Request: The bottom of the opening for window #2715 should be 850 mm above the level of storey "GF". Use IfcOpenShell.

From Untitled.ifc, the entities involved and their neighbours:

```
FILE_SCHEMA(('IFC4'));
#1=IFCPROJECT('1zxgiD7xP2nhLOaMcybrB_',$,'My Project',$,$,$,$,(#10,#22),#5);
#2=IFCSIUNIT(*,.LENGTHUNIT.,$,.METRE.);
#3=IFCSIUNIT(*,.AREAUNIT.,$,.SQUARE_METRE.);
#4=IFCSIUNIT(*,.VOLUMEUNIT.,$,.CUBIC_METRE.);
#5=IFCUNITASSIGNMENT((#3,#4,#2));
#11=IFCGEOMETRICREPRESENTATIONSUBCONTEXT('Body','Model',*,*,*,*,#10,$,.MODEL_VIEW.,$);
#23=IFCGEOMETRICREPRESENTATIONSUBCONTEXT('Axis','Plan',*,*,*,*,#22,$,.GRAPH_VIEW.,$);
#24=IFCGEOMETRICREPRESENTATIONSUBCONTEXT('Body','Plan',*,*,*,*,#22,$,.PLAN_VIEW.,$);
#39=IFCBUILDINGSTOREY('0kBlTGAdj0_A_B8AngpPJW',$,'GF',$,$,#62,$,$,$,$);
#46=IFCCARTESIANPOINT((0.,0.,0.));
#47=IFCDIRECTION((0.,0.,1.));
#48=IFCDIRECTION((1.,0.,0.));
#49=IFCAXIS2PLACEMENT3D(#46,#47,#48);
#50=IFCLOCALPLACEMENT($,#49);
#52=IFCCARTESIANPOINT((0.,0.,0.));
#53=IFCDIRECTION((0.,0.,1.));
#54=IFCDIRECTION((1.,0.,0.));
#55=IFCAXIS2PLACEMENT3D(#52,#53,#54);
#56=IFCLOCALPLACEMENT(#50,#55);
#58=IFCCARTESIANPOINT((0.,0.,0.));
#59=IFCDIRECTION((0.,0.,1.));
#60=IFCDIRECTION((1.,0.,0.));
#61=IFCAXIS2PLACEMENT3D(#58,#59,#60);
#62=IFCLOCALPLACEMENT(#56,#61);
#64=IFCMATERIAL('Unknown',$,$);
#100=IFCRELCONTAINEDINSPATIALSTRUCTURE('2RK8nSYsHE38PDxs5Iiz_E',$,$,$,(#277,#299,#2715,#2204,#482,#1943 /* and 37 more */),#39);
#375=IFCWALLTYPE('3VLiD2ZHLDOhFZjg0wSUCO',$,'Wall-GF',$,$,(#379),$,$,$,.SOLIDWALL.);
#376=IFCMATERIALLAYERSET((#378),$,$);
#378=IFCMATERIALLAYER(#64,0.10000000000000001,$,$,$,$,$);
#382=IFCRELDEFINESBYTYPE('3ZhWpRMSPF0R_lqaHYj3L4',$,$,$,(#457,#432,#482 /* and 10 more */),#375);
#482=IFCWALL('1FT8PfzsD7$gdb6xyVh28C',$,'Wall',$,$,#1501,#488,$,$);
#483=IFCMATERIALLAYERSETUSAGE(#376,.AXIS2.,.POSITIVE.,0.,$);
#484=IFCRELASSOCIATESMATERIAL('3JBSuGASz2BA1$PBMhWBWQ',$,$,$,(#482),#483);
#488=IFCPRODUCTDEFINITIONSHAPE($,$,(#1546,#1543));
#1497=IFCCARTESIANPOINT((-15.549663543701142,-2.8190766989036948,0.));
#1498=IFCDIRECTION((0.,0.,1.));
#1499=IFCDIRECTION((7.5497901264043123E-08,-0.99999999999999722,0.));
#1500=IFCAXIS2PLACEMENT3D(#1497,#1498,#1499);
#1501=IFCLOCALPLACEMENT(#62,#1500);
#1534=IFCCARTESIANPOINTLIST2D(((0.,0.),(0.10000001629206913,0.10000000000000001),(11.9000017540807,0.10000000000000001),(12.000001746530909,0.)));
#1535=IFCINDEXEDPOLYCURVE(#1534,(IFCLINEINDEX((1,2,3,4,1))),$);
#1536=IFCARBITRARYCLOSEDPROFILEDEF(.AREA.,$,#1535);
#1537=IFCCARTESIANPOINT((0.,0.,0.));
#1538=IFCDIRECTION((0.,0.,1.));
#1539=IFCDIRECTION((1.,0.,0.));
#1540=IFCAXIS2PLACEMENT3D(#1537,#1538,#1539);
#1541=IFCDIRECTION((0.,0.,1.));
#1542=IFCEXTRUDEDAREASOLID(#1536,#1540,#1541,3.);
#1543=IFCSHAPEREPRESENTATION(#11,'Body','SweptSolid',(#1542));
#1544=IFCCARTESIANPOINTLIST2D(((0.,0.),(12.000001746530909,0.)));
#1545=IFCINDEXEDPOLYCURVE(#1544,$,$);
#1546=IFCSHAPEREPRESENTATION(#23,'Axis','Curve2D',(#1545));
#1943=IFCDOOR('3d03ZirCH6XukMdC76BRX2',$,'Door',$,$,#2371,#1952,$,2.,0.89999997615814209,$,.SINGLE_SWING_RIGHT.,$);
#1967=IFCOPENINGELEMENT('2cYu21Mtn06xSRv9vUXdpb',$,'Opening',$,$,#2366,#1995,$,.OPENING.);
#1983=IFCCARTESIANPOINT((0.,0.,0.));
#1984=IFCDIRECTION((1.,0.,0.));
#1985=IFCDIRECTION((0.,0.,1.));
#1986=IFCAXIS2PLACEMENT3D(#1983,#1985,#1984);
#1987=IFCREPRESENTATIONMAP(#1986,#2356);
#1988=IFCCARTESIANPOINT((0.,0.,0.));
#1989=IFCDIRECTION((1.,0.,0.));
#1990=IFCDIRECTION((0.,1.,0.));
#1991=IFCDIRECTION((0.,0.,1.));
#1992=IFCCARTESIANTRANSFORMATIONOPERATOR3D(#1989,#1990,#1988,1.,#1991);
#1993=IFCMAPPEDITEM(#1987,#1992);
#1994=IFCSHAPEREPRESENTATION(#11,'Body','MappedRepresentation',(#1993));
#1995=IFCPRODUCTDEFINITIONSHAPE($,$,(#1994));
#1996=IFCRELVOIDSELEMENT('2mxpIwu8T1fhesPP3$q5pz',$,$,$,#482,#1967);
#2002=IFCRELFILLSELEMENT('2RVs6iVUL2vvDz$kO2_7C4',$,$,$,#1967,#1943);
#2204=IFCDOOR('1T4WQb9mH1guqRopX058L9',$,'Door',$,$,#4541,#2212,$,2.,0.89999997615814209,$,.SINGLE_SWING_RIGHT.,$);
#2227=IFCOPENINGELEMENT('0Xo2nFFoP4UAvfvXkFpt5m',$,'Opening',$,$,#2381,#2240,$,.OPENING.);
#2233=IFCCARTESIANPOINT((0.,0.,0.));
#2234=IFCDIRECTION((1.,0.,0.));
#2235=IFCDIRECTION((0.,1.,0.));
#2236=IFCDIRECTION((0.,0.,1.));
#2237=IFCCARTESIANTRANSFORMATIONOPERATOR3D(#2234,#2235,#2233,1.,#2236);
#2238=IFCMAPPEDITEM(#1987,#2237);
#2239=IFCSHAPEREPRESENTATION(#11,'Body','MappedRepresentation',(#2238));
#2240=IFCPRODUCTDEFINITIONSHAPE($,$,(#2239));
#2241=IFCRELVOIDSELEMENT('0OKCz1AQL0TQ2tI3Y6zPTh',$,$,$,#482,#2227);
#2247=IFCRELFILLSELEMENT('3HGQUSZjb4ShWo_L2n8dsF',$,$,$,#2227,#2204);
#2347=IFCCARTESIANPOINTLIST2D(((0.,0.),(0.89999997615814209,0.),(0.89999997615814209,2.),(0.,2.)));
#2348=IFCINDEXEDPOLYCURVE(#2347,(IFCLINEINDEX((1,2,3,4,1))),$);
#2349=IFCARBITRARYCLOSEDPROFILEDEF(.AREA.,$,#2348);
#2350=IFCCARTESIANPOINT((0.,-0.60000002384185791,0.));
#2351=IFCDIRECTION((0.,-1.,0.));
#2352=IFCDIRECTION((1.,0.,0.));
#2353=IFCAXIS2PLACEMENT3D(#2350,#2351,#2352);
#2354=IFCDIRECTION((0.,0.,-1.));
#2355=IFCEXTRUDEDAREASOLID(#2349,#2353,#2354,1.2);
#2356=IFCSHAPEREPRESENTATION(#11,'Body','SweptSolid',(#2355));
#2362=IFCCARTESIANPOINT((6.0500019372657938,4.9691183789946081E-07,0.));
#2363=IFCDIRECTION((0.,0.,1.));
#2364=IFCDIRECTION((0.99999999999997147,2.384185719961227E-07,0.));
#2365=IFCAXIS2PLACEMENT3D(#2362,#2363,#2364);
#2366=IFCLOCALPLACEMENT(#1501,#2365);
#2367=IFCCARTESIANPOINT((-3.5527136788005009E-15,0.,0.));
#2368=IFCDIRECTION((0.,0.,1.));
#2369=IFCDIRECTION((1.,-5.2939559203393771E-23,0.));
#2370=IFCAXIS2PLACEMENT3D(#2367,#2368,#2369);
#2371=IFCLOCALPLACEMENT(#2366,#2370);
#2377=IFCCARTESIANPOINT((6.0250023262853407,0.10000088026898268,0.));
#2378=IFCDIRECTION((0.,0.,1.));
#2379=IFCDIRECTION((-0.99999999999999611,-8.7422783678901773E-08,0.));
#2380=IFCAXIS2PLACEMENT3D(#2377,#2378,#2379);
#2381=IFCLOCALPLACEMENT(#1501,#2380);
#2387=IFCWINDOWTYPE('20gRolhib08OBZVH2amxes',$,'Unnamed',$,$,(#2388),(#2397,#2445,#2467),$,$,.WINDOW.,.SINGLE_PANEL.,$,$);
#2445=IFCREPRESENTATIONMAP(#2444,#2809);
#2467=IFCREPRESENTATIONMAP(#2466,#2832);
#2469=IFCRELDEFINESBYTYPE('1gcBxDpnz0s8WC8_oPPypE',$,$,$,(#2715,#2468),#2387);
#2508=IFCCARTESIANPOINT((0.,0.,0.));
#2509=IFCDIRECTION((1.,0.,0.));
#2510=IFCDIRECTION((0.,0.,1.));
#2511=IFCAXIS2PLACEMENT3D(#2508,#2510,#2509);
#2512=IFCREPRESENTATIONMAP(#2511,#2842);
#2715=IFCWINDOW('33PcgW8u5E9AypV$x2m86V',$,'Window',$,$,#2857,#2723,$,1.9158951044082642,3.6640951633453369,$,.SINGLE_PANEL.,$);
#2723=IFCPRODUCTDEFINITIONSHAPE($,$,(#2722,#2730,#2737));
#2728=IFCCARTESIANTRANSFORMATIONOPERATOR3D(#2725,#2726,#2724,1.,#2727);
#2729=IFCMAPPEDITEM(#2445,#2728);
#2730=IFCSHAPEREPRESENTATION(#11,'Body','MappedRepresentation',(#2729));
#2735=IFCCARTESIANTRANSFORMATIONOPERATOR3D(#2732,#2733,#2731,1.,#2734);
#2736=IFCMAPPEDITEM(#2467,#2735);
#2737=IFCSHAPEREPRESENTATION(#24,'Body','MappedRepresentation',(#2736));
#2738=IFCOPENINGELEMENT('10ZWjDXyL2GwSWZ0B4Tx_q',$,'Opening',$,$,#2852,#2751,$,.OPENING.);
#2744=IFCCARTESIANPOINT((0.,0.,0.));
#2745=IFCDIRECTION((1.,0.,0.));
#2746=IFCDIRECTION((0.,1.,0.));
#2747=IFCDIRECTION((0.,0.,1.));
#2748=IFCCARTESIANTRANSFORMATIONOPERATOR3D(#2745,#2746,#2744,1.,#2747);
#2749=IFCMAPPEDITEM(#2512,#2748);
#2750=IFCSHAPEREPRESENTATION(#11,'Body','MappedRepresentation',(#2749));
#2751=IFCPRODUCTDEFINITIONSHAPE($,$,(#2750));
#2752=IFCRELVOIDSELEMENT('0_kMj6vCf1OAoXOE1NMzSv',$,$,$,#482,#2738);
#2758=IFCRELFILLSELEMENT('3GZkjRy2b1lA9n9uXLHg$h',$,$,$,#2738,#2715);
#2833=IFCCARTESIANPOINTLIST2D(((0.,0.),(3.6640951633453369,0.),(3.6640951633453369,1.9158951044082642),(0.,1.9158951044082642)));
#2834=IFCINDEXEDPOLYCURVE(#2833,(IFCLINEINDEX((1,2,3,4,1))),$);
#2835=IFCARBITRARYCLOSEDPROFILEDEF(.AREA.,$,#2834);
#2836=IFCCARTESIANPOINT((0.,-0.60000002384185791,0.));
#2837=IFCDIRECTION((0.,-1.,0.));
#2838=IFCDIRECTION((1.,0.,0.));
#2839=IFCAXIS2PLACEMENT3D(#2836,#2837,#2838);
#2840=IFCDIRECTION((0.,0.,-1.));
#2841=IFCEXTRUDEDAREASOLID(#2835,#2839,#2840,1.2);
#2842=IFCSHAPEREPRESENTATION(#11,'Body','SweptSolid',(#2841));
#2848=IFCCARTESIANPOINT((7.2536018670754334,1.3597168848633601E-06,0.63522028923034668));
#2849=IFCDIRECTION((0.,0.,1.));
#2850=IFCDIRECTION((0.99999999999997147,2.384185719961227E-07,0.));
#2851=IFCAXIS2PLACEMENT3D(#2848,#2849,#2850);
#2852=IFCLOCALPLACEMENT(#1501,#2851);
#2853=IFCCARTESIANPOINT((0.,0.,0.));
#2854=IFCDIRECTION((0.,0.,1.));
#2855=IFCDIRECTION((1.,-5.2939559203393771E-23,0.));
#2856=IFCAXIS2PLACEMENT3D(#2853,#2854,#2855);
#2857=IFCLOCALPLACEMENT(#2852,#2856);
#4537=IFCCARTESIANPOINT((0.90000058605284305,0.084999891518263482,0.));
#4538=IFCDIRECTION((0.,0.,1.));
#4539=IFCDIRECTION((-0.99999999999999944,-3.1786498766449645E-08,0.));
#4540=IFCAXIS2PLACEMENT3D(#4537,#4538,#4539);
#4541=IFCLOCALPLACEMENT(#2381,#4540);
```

```python
import numpy as np
import ifcopenshell
import ifcopenshell.api.geometry
import ifcopenshell.geom
import ifcopenshell.util.element
import ifcopenshell.util.placement
import ifcopenshell.util.shape
import ifcopenshell.util.unit

model = ifcopenshell.open("Untitled.ifc")
unit_scale = ifcopenshell.util.unit.calculate_unit_scale(model)

window = model.by_guid("33PcgW8u5E9AypV$x2m86V")
opening = window.FillsVoids[0].RelatingOpeningElement
storey = ifcopenshell.util.element.get_container(window, ifc_class="IfcBuildingStorey")
level = ifcopenshell.util.placement.get_local_placement(storey.ObjectPlacement)[2, 3]

# The opening's origin need not be at the sill, so measure its lowest point.
shape = ifcopenshell.geom.create_shape(ifcopenshell.geom.settings(), opening)
bottom = ifcopenshell.util.shape.get_shape_bottom_elevation(shape, shape.geometry) / unit_scale
dz = level + 0.85 / unit_scale - bottom

shift = np.array([0.0, 0.0, dz])
# The window is placed relative to its opening, so it follows when the opening moves.
matrix = ifcopenshell.util.placement.get_local_placement(opening.ObjectPlacement)
matrix[:3, 3] += shift
ifcopenshell.api.geometry.edit_object_placement(
    model, product=opening, matrix=matrix, is_si=False, should_transform_children=True
)

print(f"moved by {dz * unit_scale:+.3f} m")

model.write("Untitled_updated.ifc")
```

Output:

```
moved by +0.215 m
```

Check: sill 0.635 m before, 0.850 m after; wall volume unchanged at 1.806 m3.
